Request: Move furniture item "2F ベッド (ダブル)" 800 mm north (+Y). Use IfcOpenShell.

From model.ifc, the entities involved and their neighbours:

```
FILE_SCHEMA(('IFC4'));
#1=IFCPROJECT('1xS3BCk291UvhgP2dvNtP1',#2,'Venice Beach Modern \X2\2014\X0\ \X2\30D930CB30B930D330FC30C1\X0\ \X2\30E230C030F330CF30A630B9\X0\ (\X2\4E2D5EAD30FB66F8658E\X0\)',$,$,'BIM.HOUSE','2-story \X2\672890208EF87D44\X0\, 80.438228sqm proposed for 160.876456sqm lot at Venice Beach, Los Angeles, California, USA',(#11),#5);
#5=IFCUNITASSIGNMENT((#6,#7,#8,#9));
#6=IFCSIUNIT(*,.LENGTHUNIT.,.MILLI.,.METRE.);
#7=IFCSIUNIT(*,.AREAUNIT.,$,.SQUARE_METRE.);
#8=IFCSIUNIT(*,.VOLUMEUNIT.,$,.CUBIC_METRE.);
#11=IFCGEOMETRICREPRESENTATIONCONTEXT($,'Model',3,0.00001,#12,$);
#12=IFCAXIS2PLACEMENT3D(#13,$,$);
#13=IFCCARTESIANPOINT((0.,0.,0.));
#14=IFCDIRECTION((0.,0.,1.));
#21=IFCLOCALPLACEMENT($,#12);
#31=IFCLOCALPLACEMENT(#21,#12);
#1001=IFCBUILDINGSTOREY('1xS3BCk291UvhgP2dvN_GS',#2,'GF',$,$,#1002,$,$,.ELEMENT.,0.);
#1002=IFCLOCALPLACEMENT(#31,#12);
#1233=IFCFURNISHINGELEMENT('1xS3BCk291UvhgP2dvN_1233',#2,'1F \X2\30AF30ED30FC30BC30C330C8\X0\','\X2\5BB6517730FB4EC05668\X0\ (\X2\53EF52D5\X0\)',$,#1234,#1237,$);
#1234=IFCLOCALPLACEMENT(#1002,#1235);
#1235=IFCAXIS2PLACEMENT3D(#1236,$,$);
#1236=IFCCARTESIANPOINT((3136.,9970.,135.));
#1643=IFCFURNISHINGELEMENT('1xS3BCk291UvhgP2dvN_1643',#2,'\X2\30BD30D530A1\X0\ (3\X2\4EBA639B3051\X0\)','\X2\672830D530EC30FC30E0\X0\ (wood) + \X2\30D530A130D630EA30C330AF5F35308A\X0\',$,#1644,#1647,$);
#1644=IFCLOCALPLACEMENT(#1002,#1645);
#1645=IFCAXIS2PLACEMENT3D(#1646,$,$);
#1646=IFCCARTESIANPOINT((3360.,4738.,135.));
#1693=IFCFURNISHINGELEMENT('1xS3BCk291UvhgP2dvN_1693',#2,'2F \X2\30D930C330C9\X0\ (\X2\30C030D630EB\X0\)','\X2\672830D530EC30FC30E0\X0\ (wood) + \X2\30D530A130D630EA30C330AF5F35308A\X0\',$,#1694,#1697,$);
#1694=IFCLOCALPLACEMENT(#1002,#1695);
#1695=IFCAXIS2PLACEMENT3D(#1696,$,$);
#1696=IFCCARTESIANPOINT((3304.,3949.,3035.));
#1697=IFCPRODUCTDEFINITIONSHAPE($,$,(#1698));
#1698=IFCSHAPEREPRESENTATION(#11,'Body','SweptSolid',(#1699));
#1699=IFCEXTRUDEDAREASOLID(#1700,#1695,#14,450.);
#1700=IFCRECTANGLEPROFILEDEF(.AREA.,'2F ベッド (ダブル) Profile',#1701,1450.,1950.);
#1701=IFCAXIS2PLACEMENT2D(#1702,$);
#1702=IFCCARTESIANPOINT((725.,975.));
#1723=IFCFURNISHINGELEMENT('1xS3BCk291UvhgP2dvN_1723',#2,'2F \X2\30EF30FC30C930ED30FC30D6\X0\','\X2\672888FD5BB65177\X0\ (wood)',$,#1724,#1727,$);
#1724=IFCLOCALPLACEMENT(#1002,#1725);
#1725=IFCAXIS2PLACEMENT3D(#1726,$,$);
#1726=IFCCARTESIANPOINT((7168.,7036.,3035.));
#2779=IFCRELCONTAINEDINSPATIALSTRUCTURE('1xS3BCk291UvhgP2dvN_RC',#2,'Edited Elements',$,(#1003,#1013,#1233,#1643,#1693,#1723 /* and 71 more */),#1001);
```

```python
import ifcopenshell
import ifcopenshell.api.geometry
import ifcopenshell.util.placement

model = ifcopenshell.open("model.ifc")

item = model.by_guid("1xS3BCk291UvhgP2dvN_1693")
matrix = ifcopenshell.util.placement.get_local_placement(item.ObjectPlacement)
matrix[1, 3] += 800.0
ifcopenshell.api.geometry.edit_object_placement(model, product=item, matrix=matrix, is_si=False)

print(ifcopenshell.util.placement.get_local_placement(item.ObjectPlacement).round(3) + 0.0)

model.write("model_v2.ifc")
```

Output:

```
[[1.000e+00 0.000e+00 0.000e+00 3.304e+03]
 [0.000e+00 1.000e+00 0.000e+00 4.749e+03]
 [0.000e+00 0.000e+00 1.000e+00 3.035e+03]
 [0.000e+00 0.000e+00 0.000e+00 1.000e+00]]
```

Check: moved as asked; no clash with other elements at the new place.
